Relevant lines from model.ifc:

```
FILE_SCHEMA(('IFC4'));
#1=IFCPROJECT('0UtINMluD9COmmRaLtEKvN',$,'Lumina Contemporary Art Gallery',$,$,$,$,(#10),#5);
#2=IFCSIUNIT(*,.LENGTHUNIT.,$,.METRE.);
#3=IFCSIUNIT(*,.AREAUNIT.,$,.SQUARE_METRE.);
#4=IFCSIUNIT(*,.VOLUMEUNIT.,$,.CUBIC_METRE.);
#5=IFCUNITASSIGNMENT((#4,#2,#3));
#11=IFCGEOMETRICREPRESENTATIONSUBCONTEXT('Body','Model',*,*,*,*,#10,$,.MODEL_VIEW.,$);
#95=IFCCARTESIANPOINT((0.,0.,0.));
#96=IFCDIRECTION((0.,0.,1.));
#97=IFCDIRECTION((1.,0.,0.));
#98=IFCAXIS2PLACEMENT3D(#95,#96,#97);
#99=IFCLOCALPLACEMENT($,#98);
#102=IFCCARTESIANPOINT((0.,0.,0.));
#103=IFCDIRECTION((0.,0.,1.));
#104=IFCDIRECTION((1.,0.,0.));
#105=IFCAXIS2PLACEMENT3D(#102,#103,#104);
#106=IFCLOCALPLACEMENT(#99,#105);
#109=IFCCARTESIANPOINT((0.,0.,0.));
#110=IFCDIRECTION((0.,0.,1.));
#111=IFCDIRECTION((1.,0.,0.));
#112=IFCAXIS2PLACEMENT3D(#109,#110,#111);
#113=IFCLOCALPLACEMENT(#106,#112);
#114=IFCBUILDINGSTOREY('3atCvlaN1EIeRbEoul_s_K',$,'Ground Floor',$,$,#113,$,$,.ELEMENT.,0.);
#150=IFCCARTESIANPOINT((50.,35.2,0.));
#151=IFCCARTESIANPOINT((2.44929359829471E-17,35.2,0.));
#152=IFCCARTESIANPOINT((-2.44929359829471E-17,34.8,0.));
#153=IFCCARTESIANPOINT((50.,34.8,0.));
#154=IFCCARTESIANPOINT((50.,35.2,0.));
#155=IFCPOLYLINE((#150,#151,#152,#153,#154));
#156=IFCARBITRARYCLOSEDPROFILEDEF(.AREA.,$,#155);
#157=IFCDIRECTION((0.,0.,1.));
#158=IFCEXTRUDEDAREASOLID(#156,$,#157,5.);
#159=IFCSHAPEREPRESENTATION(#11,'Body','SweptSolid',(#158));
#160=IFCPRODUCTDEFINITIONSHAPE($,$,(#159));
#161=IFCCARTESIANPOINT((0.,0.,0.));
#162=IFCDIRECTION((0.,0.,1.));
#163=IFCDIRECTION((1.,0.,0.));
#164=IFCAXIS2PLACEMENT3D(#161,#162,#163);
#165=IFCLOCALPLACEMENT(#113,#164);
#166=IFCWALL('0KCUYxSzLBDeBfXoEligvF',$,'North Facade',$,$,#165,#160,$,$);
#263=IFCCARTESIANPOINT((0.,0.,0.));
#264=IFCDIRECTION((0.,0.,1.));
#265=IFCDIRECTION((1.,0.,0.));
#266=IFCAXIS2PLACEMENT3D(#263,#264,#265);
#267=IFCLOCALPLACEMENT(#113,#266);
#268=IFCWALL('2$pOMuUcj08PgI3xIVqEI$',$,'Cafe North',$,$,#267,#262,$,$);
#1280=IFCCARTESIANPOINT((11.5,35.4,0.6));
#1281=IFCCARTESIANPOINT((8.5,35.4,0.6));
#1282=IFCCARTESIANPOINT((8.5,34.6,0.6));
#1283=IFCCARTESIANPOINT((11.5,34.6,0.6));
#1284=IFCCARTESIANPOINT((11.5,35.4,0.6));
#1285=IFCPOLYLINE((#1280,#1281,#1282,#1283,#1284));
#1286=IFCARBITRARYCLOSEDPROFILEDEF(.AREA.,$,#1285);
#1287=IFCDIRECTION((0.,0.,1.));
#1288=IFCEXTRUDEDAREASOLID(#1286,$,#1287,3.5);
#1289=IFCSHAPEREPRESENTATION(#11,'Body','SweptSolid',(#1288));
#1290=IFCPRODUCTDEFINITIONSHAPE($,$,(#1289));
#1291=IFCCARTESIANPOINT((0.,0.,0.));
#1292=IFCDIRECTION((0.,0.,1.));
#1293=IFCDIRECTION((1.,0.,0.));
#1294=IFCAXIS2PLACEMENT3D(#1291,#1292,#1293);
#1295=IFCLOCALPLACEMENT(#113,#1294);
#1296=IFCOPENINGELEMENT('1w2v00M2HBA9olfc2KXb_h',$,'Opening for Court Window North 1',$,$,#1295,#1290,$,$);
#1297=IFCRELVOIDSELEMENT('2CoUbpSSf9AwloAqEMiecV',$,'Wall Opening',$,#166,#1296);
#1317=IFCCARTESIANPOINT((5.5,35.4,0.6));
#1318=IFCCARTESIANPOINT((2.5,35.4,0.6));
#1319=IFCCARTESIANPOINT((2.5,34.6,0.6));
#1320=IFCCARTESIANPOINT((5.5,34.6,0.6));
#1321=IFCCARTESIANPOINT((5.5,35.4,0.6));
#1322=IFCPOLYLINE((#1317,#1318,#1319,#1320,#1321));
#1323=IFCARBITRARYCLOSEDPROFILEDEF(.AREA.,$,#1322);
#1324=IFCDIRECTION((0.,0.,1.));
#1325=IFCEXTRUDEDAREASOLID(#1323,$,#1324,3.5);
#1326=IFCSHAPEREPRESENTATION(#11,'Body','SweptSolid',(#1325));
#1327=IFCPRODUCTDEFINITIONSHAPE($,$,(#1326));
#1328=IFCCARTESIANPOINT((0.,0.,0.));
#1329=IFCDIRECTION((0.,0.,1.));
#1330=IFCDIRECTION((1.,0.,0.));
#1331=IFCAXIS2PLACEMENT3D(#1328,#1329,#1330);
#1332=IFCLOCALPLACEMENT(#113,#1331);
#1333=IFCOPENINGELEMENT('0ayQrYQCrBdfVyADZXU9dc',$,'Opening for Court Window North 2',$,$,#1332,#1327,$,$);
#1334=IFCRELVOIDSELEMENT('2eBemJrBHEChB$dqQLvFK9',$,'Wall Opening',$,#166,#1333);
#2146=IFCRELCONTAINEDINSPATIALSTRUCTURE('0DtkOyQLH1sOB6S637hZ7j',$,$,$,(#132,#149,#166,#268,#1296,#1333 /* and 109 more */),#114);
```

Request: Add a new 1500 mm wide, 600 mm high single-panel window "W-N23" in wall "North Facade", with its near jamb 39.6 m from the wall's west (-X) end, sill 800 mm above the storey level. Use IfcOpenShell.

```python
import numpy as np
import ifcopenshell
import ifcopenshell.api.feature
import ifcopenshell.api.geometry
import ifcopenshell.api.root
import ifcopenshell.api.spatial
import ifcopenshell.geom
import ifcopenshell.util.element
import ifcopenshell.util.placement
import ifcopenshell.util.representation
import ifcopenshell.util.shape
import ifcopenshell.util.unit

model = ifcopenshell.open("model.ifc")
unit_scale = ifcopenshell.util.unit.calculate_unit_scale(model)
settings = ifcopenshell.geom.settings()


def volume(element):
    """Net volume in cubic metres, openings subtracted."""
    shape = ifcopenshell.geom.create_shape(settings, element)
    return ifcopenshell.util.shape.get_volume(shape.geometry)


wall = model.by_guid("0KCUYxSzLBDeBfXoEligvF")
storey = ifcopenshell.util.element.get_container(wall, ifc_class="IfcBuildingStorey")
context = ifcopenshell.util.representation.get_context(model, "Model", "Body", "MODEL_VIEW")
before = volume(wall)

width, height, from_end, sill = 1.5, 0.6, 39.6, 0.8  # metres

# The wall runs along its own X axis, and the end named is its -X end.
wall_shape = ifcopenshell.geom.create_shape(settings, wall)
x, y, z = ifcopenshell.util.shape.get_vertices(wall_shape.geometry).T
start = x.min() + from_end
face, thickness = float(y.min()), float(y.max() - y.min())
wall_matrix = ifcopenshell.util.placement.get_local_placement(wall.ObjectPlacement)
level = ifcopenshell.util.placement.get_local_placement(storey.ObjectPlacement)[2, 3]


def in_wall(x, y):
    """Placement at x, y metres in the wall's axes, at sill height."""
    matrix = wall_matrix.copy()
    matrix[:, 3] = wall_matrix @ np.array([x / unit_scale, y / unit_scale, 0.0, 1.0])
    matrix[2, 3] = level + sill / unit_scale
    return matrix


# Opening: a box that overshoots both wall faces by 50 mm.
opening = ifcopenshell.api.root.create_entity(model, ifc_class="IfcOpeningElement", predefined_type="OPENING")
box = ifcopenshell.api.geometry.add_wall_representation(
    model, context=context, length=width, height=height, thickness=thickness + 0.1
)
ifcopenshell.api.geometry.assign_representation(model, product=opening, representation=box)
ifcopenshell.api.geometry.edit_object_placement(model, product=opening, matrix=in_wall(start, face - 0.05), is_si=False)
ifcopenshell.api.feature.add_feature(model, feature=opening, element=wall)

window = ifcopenshell.api.root.create_entity(model, ifc_class="IfcWindow", name="W-N23", predefined_type="WINDOW")
window.OverallWidth, window.OverallHeight = width / unit_scale, height / unit_scale
window.PartitioningType = "SINGLE_PANEL"
body = ifcopenshell.api.geometry.add_window_representation(
    model,
    context=context,
    overall_width=window.OverallWidth,
    overall_height=window.OverallHeight,
    partition_type="SINGLE_PANEL",
)
ifcopenshell.api.geometry.assign_representation(model, product=window, representation=body)
ifcopenshell.api.spatial.assign_container(model, products=[window], relating_structure=storey)
ifcopenshell.api.feature.add_filling(model, opening=opening, element=window)

# Centre the window in the wall's thickness.
ifcopenshell.api.geometry.edit_object_placement(model, product=window, matrix=in_wall(start, face), is_si=False)
window_shape = ifcopenshell.geom.create_shape(settings, window)
depth = ifcopenshell.util.shape.get_vertices(window_shape.geometry)[:, 1]
offset = face + thickness / 2 - (depth.min() + depth.max()) / 2
ifcopenshell.api.geometry.edit_object_placement(model, product=window, matrix=in_wall(start, offset), is_si=False)

after = volume(wall)

print(f"wall volume {before:.3f} -> {after:.3f} m3")

model.write("model_v2.ifc")
```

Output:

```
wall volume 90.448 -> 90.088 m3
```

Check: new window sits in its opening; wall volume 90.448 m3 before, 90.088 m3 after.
